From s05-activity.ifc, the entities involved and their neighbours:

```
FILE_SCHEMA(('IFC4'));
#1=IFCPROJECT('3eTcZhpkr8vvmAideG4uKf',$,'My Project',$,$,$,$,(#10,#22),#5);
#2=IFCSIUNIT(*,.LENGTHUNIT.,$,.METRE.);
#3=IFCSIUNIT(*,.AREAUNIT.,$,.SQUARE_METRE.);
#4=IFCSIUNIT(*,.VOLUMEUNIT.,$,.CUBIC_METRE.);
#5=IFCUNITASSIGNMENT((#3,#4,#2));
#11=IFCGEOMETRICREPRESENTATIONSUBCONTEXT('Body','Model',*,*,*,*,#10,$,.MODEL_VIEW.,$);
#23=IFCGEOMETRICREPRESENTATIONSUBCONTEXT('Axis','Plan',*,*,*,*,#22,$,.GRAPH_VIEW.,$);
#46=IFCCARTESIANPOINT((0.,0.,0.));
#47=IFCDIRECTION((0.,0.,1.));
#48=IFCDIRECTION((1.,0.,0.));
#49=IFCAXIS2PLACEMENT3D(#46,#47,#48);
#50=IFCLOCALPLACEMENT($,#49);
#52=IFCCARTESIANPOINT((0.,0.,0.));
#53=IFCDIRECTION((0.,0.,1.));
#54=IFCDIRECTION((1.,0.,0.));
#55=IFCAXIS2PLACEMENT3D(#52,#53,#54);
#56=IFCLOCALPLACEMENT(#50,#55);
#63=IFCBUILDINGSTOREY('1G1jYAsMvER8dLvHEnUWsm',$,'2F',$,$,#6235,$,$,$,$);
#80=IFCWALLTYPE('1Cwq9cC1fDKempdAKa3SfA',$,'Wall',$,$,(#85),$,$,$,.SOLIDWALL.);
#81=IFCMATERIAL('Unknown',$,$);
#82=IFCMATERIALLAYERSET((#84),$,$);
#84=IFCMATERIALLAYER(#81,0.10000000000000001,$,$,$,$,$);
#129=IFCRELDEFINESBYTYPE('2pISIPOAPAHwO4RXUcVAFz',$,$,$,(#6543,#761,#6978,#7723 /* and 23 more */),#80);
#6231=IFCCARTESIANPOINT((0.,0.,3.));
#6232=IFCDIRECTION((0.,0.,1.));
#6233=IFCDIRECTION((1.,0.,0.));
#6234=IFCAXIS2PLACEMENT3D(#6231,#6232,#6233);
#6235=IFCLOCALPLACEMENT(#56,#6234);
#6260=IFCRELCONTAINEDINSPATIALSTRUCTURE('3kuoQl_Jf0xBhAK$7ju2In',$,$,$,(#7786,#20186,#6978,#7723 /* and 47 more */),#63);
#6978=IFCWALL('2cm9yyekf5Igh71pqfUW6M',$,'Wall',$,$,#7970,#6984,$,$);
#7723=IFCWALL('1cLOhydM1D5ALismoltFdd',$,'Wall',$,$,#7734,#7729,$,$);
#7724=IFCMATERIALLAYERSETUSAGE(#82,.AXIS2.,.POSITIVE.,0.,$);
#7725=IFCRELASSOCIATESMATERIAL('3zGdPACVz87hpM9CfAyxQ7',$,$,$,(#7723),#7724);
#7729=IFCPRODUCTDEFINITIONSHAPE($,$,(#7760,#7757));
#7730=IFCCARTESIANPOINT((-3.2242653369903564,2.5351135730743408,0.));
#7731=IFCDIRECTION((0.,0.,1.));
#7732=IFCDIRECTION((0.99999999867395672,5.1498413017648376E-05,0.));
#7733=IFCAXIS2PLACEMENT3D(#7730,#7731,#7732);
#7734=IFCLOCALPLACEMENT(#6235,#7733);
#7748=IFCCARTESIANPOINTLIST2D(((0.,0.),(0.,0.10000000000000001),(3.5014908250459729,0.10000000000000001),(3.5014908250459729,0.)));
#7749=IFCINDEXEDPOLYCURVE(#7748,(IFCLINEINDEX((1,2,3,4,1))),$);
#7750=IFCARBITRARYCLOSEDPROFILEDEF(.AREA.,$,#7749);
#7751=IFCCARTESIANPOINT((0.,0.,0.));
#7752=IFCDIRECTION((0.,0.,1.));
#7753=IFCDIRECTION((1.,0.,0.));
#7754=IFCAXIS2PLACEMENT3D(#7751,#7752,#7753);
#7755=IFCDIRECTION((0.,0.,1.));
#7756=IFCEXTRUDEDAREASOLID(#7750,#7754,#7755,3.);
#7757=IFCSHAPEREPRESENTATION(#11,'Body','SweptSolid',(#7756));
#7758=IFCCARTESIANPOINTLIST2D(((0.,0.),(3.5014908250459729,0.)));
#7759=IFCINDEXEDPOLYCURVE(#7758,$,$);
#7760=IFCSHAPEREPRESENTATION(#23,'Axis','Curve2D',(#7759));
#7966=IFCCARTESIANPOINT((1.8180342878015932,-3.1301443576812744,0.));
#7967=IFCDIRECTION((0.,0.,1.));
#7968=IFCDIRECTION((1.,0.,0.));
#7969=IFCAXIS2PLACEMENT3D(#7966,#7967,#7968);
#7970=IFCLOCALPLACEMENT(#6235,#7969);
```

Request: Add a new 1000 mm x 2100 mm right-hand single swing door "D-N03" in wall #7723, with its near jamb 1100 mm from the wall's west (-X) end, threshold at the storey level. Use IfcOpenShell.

```python
import numpy as np
import ifcopenshell
import ifcopenshell.api.feature
import ifcopenshell.api.geometry
import ifcopenshell.api.root
import ifcopenshell.api.spatial
import ifcopenshell.geom
import ifcopenshell.util.element
import ifcopenshell.util.placement
import ifcopenshell.util.representation
import ifcopenshell.util.shape
import ifcopenshell.util.unit

model = ifcopenshell.open("s05-activity.ifc")
unit_scale = ifcopenshell.util.unit.calculate_unit_scale(model)
settings = ifcopenshell.geom.settings()


def volume(element):
    """Net volume in cubic metres, openings subtracted."""
    shape = ifcopenshell.geom.create_shape(settings, element)
    return ifcopenshell.util.shape.get_volume(shape.geometry)


wall = model.by_guid("1cLOhydM1D5ALismoltFdd")
storey = ifcopenshell.util.element.get_container(wall, ifc_class="IfcBuildingStorey")
context = ifcopenshell.util.representation.get_context(model, "Model", "Body", "MODEL_VIEW")
before = volume(wall)

width, height, from_end, sill = 1, 2.1, 1.1, 0.0  # metres

# The wall runs along its own X axis, and the end named is its -X end.
wall_shape = ifcopenshell.geom.create_shape(settings, wall)
x, y, z = ifcopenshell.util.shape.get_vertices(wall_shape.geometry).T
start = x.min() + from_end
face, thickness = float(y.min()), float(y.max() - y.min())
wall_matrix = ifcopenshell.util.placement.get_local_placement(wall.ObjectPlacement)
level = ifcopenshell.util.placement.get_local_placement(storey.ObjectPlacement)[2, 3]


def in_wall(x, y):
    """Placement at x, y metres in the wall's axes, at sill height."""
    matrix = wall_matrix.copy()
    matrix[:, 3] = wall_matrix @ np.array([x / unit_scale, y / unit_scale, 0.0, 1.0])
    matrix[2, 3] = level + sill / unit_scale
    return matrix


# Opening: a box that overshoots both wall faces by 50 mm.
opening = ifcopenshell.api.root.create_entity(model, ifc_class="IfcOpeningElement", predefined_type="OPENING")
box = ifcopenshell.api.geometry.add_wall_representation(
    model, context=context, length=width, height=height, thickness=thickness + 0.1
)
ifcopenshell.api.geometry.assign_representation(model, product=opening, representation=box)
ifcopenshell.api.geometry.edit_object_placement(model, product=opening, matrix=in_wall(start, face - 0.05), is_si=False)
ifcopenshell.api.feature.add_feature(model, feature=opening, element=wall)

door = ifcopenshell.api.root.create_entity(model, ifc_class="IfcDoor", name="D-N03", predefined_type="DOOR")
door.OverallWidth, door.OverallHeight = width / unit_scale, height / unit_scale
door.OperationType = "SINGLE_SWING_RIGHT"
body = ifcopenshell.api.geometry.add_door_representation(
    model,
    context=context,
    overall_width=door.OverallWidth,
    overall_height=door.OverallHeight,
    operation_type="SINGLE_SWING_RIGHT",
    lining_properties={"LiningDepth": thickness / unit_scale, "ThresholdDepth": thickness / unit_scale},
)
ifcopenshell.api.geometry.assign_representation(model, product=door, representation=body)
ifcopenshell.api.spatial.assign_container(model, products=[door], relating_structure=storey)
ifcopenshell.api.feature.add_filling(model, opening=opening, element=door)

# The lining spans the wall, so the door starts at the wall face.
ifcopenshell.api.geometry.edit_object_placement(model, product=door, matrix=in_wall(start, face), is_si=False)

after = volume(wall)

print(f"wall volume {before:.3f} -> {after:.3f} m3")

model.write("s05-activity_v2.ifc")
```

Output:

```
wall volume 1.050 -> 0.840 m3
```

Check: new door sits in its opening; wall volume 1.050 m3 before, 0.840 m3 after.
